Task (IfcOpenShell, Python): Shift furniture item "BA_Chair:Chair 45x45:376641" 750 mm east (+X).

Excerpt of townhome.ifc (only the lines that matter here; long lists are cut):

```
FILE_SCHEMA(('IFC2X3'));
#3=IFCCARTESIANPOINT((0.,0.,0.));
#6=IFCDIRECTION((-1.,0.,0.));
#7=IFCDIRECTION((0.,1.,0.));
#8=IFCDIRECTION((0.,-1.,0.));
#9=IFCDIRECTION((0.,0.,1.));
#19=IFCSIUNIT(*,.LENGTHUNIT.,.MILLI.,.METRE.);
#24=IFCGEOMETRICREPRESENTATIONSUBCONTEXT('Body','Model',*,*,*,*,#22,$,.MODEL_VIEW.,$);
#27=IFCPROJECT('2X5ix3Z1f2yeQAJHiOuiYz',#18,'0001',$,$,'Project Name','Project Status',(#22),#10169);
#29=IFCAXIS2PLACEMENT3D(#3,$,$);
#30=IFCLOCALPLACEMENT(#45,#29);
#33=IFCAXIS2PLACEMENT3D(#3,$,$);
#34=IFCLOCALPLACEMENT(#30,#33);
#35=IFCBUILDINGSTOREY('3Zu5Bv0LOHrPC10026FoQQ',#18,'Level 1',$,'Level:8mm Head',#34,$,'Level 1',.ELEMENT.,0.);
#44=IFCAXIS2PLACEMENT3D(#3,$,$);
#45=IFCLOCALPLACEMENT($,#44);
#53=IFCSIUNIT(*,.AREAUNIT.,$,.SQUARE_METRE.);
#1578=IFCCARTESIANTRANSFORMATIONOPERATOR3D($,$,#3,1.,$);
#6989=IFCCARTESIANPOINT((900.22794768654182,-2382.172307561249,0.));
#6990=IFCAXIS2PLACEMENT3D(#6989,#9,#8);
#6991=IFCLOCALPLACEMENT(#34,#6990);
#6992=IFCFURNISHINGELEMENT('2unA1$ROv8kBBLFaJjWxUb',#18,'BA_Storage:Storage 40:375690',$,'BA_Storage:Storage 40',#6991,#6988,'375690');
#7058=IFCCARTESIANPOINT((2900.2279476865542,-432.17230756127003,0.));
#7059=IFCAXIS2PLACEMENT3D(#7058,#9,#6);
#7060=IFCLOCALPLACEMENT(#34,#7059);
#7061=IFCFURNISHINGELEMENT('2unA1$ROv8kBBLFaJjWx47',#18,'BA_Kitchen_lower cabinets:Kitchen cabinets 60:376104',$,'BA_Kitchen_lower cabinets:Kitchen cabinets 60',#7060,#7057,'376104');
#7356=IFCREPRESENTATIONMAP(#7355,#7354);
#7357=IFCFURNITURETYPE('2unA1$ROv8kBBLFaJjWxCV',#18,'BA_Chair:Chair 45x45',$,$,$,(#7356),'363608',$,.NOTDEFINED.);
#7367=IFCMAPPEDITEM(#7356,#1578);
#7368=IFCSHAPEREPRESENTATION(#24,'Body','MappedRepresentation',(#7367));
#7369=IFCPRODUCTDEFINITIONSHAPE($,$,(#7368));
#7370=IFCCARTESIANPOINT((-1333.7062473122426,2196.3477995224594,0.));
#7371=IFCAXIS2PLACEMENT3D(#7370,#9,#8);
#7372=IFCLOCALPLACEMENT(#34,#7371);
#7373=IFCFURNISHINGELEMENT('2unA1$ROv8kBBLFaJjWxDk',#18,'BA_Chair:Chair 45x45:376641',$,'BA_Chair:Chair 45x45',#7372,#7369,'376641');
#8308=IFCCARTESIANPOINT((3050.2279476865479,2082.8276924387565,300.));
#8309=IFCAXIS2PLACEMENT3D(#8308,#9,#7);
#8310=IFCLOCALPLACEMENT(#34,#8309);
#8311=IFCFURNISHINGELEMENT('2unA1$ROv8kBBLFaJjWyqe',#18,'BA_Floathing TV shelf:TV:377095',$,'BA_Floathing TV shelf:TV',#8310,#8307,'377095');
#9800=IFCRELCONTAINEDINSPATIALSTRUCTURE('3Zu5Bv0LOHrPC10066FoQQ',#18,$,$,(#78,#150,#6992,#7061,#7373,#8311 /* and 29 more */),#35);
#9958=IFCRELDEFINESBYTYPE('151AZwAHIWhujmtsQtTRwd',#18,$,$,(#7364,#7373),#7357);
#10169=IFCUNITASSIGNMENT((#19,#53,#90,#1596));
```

```python
import ifcopenshell
import ifcopenshell.api.geometry
import ifcopenshell.util.placement
import ifcopenshell.util.unit

model = ifcopenshell.open("townhome.ifc")
unit_scale = ifcopenshell.util.unit.calculate_unit_scale(model)

item = model.by_guid("2unA1$ROv8kBBLFaJjWxDk")
matrix = ifcopenshell.util.placement.get_local_placement(item.ObjectPlacement)
matrix[0, 3] += 0.75 / unit_scale
ifcopenshell.api.geometry.edit_object_placement(model, product=item, matrix=matrix, is_si=False)

print(ifcopenshell.util.placement.get_local_placement(item.ObjectPlacement).round(3) + 0.0)

model.write("townhome_edited.ifc")
```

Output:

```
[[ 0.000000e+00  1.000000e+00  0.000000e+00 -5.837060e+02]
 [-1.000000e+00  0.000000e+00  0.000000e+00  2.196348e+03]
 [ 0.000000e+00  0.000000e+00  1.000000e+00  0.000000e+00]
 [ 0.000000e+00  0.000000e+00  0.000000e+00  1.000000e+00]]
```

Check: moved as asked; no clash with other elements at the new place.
